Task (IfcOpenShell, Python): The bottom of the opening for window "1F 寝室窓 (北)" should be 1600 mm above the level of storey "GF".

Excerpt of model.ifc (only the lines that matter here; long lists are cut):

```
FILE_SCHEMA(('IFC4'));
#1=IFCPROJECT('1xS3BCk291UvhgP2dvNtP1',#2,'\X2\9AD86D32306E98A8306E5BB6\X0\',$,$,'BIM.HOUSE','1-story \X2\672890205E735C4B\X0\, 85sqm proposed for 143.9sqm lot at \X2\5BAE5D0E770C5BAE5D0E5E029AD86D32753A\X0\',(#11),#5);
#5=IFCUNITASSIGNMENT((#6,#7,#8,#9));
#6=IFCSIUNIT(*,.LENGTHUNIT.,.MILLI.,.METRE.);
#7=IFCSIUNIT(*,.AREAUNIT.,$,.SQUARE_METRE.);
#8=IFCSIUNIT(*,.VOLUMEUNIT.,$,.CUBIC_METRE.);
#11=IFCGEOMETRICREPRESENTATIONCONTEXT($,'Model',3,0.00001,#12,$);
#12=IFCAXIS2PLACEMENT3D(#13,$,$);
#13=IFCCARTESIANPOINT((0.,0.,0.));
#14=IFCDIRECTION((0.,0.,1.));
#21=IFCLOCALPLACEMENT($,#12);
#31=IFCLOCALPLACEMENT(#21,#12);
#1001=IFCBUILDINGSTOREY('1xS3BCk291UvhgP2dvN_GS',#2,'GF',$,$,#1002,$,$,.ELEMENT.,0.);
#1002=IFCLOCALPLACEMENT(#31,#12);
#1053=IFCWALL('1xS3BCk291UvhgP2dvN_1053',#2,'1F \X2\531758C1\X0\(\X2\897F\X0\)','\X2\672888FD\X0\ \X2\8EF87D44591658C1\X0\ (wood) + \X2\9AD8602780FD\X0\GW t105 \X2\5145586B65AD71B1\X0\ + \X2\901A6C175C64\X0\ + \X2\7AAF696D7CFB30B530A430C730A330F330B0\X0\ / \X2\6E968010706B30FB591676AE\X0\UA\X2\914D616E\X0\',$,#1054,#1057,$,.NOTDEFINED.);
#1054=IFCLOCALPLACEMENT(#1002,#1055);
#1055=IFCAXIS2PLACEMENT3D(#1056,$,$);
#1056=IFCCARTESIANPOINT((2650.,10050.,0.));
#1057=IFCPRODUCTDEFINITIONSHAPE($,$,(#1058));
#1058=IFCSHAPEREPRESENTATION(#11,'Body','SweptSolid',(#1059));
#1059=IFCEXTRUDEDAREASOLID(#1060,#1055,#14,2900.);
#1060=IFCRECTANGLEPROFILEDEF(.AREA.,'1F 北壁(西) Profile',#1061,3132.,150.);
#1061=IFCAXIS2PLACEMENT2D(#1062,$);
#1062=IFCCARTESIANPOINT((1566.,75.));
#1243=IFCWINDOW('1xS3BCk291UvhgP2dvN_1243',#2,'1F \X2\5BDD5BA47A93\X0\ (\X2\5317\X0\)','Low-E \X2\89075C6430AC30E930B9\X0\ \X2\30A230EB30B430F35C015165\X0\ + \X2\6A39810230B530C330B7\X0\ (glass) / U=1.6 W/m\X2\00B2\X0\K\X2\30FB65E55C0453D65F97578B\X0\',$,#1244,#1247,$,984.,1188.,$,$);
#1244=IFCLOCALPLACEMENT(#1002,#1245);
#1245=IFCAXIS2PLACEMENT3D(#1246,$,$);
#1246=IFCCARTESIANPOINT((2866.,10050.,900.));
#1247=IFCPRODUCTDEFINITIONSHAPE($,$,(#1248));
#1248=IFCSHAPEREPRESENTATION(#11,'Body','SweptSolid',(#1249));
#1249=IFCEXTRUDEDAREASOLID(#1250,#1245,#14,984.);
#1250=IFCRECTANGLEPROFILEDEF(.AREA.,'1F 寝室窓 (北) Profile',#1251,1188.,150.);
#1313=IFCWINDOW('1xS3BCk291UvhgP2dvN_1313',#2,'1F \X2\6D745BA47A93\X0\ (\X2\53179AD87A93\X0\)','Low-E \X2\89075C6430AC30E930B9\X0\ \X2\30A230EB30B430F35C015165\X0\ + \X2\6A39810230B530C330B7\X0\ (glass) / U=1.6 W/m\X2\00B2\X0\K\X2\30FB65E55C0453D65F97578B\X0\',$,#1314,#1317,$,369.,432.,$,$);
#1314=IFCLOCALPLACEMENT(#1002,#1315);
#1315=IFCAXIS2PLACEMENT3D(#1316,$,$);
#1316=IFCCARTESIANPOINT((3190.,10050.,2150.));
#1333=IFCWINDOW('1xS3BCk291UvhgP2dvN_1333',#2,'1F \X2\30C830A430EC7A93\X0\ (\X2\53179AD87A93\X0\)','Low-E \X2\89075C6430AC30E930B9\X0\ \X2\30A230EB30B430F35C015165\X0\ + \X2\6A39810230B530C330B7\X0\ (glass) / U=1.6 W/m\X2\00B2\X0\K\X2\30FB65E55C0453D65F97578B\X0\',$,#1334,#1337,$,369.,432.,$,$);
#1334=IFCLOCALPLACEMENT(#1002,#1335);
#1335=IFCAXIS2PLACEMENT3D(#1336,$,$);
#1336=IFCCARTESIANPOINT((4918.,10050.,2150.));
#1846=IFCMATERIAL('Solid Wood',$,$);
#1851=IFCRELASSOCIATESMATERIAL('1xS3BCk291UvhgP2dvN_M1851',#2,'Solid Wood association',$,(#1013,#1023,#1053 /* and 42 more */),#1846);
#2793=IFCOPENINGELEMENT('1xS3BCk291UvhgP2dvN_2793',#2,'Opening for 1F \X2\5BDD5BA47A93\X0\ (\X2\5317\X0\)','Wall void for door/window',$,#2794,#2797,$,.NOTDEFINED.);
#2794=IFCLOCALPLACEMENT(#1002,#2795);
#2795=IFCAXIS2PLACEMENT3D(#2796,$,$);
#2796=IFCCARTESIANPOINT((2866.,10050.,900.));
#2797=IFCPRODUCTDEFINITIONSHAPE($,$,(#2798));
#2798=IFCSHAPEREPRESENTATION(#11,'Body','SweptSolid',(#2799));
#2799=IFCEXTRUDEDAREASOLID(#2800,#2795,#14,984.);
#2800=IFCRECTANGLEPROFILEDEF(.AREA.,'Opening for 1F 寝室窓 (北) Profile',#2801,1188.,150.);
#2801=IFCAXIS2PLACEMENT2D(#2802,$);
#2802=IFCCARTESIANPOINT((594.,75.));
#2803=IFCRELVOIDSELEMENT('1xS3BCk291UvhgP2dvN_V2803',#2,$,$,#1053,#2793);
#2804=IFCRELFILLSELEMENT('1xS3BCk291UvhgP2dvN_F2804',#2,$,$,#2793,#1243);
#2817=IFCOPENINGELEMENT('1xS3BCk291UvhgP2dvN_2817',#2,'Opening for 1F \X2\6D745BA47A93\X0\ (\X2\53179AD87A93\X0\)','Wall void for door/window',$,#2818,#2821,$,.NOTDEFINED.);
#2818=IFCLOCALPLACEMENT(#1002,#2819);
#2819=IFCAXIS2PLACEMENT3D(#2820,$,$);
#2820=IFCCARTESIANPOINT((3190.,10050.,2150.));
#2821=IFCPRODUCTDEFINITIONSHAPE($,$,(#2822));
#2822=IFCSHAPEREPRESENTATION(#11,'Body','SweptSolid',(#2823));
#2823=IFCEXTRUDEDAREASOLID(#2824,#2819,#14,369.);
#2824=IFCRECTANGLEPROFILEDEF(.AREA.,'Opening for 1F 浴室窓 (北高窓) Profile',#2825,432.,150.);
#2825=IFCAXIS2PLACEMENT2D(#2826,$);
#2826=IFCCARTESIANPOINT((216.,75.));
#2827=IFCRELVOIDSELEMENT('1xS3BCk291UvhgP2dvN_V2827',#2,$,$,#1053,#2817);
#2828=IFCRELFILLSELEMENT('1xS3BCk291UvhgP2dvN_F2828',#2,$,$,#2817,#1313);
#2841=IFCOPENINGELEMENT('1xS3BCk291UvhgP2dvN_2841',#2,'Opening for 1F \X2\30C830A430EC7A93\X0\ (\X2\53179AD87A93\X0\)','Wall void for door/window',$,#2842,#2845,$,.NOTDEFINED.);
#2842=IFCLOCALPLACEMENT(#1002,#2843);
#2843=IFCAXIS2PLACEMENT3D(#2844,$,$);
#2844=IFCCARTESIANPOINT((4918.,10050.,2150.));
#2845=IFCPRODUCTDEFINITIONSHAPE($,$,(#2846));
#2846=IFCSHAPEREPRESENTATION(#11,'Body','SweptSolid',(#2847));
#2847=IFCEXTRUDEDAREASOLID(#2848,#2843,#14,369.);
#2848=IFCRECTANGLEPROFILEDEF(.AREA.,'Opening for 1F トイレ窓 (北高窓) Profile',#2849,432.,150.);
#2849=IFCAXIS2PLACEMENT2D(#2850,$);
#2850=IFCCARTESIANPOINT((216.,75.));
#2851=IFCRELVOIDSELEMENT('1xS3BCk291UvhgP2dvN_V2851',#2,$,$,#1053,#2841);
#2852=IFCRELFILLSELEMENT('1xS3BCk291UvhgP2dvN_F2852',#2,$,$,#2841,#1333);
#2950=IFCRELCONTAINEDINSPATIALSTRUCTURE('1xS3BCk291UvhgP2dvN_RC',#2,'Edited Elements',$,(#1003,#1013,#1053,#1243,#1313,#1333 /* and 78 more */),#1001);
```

```python
import numpy as np
import ifcopenshell
import ifcopenshell.api.geometry
import ifcopenshell.geom
import ifcopenshell.util.element
import ifcopenshell.util.placement
import ifcopenshell.util.shape
import ifcopenshell.util.unit

model = ifcopenshell.open("model.ifc")
unit_scale = ifcopenshell.util.unit.calculate_unit_scale(model)

window = model.by_guid("1xS3BCk291UvhgP2dvN_1243")
opening = window.FillsVoids[0].RelatingOpeningElement
storey = ifcopenshell.util.element.get_container(window, ifc_class="IfcBuildingStorey")
level = ifcopenshell.util.placement.get_local_placement(storey.ObjectPlacement)[2, 3]

# The opening's origin need not be at the sill, so measure its lowest point.
shape = ifcopenshell.geom.create_shape(ifcopenshell.geom.settings(), opening)
bottom = ifcopenshell.util.shape.get_shape_bottom_elevation(shape, shape.geometry) / unit_scale
dz = level + 1600.0 - bottom

shift = np.array([0.0, 0.0, dz])
# The window is not placed relative to its opening, so move both.
for product in (opening, window):
    matrix = ifcopenshell.util.placement.get_local_placement(product.ObjectPlacement)
    matrix[:3, 3] += shift
    ifcopenshell.api.geometry.edit_object_placement(model, product=product, matrix=matrix, is_si=False)

print(f"moved by {dz * unit_scale:+.3f} m")

model.write("model_updated.ifc")
```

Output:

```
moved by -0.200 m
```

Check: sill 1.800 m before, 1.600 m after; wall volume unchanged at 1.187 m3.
